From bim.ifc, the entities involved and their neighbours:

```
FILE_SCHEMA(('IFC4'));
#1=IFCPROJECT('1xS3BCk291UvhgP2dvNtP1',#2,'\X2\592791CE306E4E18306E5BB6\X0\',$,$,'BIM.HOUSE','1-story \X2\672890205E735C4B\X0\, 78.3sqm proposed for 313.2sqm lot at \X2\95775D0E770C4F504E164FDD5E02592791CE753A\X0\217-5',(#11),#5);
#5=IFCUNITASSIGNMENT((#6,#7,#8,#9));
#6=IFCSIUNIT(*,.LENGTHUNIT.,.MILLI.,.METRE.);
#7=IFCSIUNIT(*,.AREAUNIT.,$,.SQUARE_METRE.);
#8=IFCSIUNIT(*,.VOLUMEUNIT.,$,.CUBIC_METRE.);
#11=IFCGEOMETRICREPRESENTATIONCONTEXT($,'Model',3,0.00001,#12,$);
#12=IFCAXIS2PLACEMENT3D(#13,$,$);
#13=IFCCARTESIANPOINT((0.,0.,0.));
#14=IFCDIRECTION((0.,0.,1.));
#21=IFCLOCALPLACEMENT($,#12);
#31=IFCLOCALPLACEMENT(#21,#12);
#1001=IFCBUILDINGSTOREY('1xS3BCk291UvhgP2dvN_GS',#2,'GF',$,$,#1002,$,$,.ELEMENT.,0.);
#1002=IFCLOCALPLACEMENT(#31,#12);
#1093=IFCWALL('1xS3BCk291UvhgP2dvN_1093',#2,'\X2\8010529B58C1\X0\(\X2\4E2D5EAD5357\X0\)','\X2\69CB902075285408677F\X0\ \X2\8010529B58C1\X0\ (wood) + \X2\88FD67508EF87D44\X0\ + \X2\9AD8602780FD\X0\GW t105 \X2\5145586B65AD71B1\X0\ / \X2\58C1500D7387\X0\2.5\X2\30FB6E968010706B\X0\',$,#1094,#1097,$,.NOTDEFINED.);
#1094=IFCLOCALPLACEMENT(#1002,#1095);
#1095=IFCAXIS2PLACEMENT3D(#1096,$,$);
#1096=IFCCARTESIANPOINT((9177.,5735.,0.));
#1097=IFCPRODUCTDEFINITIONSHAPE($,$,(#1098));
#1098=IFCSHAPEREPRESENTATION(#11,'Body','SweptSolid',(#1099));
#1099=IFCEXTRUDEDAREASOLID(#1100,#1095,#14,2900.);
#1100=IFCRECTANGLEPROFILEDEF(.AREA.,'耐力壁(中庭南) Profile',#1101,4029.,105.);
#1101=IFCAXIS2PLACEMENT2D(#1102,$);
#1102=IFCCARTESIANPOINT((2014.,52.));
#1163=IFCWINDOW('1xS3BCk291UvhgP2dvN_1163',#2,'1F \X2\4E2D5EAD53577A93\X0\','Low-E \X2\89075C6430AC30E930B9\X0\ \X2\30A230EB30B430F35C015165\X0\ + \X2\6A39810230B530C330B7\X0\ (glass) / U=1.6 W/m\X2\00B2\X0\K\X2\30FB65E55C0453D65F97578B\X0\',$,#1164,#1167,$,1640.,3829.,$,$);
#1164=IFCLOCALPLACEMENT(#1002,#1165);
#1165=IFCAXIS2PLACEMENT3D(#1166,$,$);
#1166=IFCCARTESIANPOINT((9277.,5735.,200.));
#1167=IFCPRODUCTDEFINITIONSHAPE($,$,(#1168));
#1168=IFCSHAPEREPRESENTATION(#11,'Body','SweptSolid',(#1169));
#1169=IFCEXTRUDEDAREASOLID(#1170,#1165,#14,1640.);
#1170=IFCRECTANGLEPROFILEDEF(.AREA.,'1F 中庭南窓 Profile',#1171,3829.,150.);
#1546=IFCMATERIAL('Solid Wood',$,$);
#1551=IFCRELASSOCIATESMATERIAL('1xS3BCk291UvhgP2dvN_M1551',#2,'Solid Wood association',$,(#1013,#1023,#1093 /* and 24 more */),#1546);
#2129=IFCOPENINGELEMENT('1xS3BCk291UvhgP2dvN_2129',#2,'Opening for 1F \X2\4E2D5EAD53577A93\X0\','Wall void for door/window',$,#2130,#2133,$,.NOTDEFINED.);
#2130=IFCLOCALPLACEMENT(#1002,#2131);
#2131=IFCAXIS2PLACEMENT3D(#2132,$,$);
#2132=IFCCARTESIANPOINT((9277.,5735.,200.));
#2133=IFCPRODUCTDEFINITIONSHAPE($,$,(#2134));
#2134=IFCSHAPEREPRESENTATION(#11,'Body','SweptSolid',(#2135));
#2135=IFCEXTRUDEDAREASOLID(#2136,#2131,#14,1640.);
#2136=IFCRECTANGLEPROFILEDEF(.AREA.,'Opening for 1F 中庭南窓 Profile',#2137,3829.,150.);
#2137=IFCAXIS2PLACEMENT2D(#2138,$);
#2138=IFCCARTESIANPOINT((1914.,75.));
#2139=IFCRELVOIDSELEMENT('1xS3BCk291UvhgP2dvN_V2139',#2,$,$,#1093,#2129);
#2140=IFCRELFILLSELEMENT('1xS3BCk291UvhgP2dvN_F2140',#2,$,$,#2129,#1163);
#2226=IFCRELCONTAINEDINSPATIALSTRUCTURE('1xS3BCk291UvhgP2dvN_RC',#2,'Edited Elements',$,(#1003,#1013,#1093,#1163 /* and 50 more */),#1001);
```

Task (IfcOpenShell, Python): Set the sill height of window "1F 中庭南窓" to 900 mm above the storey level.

```python
import numpy as np
import ifcopenshell
import ifcopenshell.api.geometry
import ifcopenshell.geom
import ifcopenshell.util.element
import ifcopenshell.util.placement
import ifcopenshell.util.shape
import ifcopenshell.util.unit

model = ifcopenshell.open("bim.ifc")
unit_scale = ifcopenshell.util.unit.calculate_unit_scale(model)

window = model.by_guid("1xS3BCk291UvhgP2dvN_1163")
opening = window.FillsVoids[0].RelatingOpeningElement
storey = ifcopenshell.util.element.get_container(window, ifc_class="IfcBuildingStorey")
level = ifcopenshell.util.placement.get_local_placement(storey.ObjectPlacement)[2, 3]

# The opening's origin need not be at the sill, so measure its lowest point.
shape = ifcopenshell.geom.create_shape(ifcopenshell.geom.settings(), opening)
bottom = ifcopenshell.util.shape.get_shape_bottom_elevation(shape, shape.geometry) / unit_scale
dz = level + 0.9 / unit_scale - bottom

shift = np.array([0.0, 0.0, dz])
# The window is not placed relative to its opening, so move both.
for product in (opening, window):
    matrix = ifcopenshell.util.placement.get_local_placement(product.ObjectPlacement)
    matrix[:3, 3] += shift
    ifcopenshell.api.geometry.edit_object_placement(model, product=product, matrix=matrix, is_si=False)

print(f"moved by {dz * unit_scale:+.3f} m")

model.write("bim_v2.ifc")
```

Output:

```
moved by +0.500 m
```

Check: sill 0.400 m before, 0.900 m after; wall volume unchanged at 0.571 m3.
